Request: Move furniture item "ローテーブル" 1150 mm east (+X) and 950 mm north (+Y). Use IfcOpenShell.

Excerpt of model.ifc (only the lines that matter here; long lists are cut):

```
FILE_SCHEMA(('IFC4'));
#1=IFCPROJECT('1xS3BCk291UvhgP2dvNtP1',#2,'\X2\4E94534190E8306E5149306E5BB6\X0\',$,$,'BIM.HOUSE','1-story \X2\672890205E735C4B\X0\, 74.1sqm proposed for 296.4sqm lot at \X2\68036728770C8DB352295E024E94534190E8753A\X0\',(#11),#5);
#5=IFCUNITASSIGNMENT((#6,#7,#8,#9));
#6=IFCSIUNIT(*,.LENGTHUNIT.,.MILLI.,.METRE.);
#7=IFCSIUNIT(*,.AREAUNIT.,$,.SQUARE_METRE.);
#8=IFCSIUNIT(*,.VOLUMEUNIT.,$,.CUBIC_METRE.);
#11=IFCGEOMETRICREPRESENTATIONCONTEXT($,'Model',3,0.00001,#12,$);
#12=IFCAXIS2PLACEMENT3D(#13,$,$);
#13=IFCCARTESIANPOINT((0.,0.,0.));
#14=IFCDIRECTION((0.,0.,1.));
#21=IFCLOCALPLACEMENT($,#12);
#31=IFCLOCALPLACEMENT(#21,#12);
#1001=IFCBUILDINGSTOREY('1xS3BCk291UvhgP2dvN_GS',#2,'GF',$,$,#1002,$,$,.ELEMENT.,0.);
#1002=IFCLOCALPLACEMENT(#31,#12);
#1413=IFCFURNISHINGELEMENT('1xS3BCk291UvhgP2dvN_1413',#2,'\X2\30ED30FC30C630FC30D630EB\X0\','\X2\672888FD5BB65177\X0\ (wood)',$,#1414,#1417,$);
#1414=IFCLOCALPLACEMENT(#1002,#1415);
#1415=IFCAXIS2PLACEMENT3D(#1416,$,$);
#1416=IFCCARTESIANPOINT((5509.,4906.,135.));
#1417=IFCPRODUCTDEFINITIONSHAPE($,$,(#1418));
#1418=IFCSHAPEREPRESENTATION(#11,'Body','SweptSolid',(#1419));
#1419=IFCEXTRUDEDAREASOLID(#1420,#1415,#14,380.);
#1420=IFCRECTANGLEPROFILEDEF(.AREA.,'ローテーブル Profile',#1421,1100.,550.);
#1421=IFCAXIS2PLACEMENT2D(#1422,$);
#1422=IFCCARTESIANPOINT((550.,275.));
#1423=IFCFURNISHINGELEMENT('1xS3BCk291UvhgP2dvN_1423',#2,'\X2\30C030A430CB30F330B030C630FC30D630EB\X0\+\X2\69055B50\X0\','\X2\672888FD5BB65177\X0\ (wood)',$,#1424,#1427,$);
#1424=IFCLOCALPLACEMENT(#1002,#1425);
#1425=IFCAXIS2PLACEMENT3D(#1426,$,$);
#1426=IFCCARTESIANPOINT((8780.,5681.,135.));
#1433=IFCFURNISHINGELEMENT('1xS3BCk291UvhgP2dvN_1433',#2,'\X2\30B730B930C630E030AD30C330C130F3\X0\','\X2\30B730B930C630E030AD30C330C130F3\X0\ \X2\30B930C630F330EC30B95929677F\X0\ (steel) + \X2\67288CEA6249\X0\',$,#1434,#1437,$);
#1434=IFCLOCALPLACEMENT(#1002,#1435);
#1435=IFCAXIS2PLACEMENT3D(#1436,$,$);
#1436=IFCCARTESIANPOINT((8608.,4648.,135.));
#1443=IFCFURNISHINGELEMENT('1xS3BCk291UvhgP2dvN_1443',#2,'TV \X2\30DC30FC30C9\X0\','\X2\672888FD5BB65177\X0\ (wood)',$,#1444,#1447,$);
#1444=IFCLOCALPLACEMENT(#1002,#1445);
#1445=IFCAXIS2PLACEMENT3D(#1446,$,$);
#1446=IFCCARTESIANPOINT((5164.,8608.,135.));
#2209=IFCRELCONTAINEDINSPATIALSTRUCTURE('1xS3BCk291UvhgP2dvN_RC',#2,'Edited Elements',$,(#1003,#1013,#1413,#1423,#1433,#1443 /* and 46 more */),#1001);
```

```python
import ifcopenshell
import ifcopenshell.api.geometry
import ifcopenshell.util.placement
import ifcopenshell.util.unit

model = ifcopenshell.open("model.ifc")
unit_scale = ifcopenshell.util.unit.calculate_unit_scale(model)

item = model.by_guid("1xS3BCk291UvhgP2dvN_1413")
matrix = ifcopenshell.util.placement.get_local_placement(item.ObjectPlacement)
matrix[0, 3] += 1.15 / unit_scale
matrix[1, 3] += 0.95 / unit_scale
ifcopenshell.api.geometry.edit_object_placement(model, product=item, matrix=matrix, is_si=False)

print(ifcopenshell.util.placement.get_local_placement(item.ObjectPlacement).round(3) + 0.0)

model.write("model_edited.ifc")
```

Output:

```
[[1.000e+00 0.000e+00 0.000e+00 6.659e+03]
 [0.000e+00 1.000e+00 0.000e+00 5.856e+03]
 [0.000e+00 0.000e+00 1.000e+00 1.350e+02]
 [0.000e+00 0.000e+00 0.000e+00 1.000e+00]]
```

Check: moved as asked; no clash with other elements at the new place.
